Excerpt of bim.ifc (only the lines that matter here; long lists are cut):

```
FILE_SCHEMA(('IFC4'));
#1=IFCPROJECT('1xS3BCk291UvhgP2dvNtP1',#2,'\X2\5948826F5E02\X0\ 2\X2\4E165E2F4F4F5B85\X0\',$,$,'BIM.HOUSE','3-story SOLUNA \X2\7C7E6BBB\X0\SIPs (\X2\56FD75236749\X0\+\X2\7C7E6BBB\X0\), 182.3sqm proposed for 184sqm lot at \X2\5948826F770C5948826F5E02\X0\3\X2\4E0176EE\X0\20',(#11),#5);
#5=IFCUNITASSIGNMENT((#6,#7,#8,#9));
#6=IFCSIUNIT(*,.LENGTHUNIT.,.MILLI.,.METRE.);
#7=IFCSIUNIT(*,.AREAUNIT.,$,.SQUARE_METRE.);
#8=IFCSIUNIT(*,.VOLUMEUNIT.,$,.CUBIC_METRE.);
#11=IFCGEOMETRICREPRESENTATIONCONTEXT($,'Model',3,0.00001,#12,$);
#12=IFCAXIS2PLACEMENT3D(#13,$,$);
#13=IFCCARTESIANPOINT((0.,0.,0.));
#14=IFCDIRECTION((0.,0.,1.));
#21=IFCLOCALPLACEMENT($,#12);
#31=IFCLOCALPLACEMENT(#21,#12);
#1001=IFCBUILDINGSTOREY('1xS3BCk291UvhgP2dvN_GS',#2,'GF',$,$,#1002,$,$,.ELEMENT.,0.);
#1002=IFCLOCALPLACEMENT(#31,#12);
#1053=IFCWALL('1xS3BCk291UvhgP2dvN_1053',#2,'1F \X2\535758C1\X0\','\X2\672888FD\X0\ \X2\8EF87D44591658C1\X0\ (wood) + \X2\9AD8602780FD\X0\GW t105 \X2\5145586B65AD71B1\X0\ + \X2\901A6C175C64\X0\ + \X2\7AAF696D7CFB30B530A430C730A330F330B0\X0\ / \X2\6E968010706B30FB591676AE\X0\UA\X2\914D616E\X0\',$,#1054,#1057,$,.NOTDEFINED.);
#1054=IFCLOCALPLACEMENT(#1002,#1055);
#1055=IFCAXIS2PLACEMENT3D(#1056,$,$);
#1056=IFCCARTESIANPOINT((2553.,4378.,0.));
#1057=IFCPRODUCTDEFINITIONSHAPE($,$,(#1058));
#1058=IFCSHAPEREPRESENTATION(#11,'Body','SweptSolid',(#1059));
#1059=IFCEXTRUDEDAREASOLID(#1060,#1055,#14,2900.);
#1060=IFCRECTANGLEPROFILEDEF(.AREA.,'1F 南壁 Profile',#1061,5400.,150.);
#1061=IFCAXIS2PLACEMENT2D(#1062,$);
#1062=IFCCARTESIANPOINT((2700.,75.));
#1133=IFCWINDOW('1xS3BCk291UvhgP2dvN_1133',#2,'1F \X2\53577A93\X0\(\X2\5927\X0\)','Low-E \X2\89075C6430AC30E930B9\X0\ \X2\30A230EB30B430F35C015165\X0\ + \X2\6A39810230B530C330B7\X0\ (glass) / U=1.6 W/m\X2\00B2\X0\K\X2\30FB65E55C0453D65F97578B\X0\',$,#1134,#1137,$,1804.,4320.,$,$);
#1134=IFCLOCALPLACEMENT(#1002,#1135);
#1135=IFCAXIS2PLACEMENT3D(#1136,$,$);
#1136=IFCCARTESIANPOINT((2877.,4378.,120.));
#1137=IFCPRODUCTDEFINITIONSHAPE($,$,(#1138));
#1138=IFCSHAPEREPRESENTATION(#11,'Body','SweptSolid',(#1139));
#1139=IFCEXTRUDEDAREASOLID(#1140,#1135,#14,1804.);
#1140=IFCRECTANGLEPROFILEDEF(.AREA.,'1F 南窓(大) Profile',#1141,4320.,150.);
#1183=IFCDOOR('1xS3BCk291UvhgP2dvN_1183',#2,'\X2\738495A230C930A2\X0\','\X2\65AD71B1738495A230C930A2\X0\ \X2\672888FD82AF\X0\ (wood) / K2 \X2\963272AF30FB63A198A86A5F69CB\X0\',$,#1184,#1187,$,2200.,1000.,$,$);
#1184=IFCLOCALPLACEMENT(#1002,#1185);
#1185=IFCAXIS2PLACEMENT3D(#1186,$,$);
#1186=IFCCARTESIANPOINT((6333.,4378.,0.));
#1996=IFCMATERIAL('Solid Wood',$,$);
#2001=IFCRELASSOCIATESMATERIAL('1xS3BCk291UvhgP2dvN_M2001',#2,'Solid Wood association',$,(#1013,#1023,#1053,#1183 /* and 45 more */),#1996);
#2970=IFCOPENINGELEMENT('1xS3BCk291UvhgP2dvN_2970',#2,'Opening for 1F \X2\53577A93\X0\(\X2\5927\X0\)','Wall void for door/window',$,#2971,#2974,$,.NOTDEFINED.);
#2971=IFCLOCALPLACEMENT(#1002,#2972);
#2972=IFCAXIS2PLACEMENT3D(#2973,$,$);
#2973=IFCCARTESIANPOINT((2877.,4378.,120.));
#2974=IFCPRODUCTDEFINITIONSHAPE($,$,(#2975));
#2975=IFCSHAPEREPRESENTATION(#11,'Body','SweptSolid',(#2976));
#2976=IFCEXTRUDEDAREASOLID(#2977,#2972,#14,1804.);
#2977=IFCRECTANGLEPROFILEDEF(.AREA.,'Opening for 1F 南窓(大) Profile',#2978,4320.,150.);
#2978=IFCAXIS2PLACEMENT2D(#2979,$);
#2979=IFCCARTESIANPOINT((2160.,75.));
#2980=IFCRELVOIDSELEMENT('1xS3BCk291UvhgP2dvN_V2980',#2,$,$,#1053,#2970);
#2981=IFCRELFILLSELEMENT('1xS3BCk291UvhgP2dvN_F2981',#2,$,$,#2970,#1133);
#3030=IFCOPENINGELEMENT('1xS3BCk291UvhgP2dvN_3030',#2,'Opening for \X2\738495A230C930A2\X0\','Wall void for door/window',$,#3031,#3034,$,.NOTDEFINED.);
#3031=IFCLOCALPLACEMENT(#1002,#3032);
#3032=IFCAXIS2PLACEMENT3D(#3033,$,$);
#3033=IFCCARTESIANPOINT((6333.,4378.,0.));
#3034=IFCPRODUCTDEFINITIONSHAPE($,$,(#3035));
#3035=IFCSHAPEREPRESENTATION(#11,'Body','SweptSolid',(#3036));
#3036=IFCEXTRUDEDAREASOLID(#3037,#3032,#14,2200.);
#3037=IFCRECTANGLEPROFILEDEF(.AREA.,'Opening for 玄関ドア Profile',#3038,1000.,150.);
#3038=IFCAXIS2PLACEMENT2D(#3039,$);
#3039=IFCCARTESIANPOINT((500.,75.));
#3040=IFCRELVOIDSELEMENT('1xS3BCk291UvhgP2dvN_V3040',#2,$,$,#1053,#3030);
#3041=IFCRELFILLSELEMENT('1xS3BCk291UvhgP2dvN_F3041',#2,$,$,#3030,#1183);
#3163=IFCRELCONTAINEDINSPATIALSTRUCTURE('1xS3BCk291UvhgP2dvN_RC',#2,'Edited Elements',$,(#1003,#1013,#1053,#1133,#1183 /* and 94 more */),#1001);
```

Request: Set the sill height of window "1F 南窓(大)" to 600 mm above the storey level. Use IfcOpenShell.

```python
import numpy as np
import ifcopenshell
import ifcopenshell.api.geometry
import ifcopenshell.geom
import ifcopenshell.util.element
import ifcopenshell.util.placement
import ifcopenshell.util.shape
import ifcopenshell.util.unit

model = ifcopenshell.open("bim.ifc")
unit_scale = ifcopenshell.util.unit.calculate_unit_scale(model)

window = model.by_guid("1xS3BCk291UvhgP2dvN_1133")
opening = window.FillsVoids[0].RelatingOpeningElement
storey = ifcopenshell.util.element.get_container(window, ifc_class="IfcBuildingStorey")
level = ifcopenshell.util.placement.get_local_placement(storey.ObjectPlacement)[2, 3]

# The opening's origin need not be at the sill, so measure its lowest point.
shape = ifcopenshell.geom.create_shape(ifcopenshell.geom.settings(), opening)
bottom = ifcopenshell.util.shape.get_shape_bottom_elevation(shape, shape.geometry) / unit_scale
dz = level + 0.6 / unit_scale - bottom

shift = np.array([0.0, 0.0, dz])
# The window is not placed relative to its opening, so move both.
for product in (opening, window):
    matrix = ifcopenshell.util.placement.get_local_placement(product.ObjectPlacement)
    matrix[:3, 3] += shift
    ifcopenshell.api.geometry.edit_object_placement(model, product=product, matrix=matrix, is_si=False)

print(f"moved by {dz * unit_scale:+.3f} m")

model.write("bim_v2.ifc")
```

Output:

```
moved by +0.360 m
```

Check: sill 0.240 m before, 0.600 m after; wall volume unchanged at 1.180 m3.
